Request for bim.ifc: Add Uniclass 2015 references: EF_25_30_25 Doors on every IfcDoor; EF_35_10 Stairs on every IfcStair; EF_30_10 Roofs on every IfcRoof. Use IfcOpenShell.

First a look at what the model holds.

```python
import ifcopenshell

model = ifcopenshell.open("bim.ifc")
print(model.schema)
print("classifications:", [c.Name for c in model.by_type("IfcClassification")])
for ifc_class in ("IfcDoor", "IfcRoof", "IfcStair", "IfcWall", "IfcWindow"):
    print(ifc_class, len(model.by_type(ifc_class)))
```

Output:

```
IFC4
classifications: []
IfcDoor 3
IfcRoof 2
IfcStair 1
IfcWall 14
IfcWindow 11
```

```python
import ifcopenshell
import ifcopenshell.api.classification

model = ifcopenshell.open("bim.ifc")

system = ifcopenshell.api.classification.add_classification(model, classification="Uniclass 2015")

codes = {
    "IfcDoor": ("EF_25_30_25", "Doors"),
    "IfcStair": ("EF_35_10", "Stairs"),
    "IfcRoof": ("EF_30_10", "Roofs"),
}
for ifc_class, (code, name) in codes.items():
    products = model.by_type(ifc_class)
    ifcopenshell.api.classification.add_reference(
        model, products=products, classification=system, identification=code, name=name
    )
    print(code, len(products))

model.write("bim_edited.ifc")
```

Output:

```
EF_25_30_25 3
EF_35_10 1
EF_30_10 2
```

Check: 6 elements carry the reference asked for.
